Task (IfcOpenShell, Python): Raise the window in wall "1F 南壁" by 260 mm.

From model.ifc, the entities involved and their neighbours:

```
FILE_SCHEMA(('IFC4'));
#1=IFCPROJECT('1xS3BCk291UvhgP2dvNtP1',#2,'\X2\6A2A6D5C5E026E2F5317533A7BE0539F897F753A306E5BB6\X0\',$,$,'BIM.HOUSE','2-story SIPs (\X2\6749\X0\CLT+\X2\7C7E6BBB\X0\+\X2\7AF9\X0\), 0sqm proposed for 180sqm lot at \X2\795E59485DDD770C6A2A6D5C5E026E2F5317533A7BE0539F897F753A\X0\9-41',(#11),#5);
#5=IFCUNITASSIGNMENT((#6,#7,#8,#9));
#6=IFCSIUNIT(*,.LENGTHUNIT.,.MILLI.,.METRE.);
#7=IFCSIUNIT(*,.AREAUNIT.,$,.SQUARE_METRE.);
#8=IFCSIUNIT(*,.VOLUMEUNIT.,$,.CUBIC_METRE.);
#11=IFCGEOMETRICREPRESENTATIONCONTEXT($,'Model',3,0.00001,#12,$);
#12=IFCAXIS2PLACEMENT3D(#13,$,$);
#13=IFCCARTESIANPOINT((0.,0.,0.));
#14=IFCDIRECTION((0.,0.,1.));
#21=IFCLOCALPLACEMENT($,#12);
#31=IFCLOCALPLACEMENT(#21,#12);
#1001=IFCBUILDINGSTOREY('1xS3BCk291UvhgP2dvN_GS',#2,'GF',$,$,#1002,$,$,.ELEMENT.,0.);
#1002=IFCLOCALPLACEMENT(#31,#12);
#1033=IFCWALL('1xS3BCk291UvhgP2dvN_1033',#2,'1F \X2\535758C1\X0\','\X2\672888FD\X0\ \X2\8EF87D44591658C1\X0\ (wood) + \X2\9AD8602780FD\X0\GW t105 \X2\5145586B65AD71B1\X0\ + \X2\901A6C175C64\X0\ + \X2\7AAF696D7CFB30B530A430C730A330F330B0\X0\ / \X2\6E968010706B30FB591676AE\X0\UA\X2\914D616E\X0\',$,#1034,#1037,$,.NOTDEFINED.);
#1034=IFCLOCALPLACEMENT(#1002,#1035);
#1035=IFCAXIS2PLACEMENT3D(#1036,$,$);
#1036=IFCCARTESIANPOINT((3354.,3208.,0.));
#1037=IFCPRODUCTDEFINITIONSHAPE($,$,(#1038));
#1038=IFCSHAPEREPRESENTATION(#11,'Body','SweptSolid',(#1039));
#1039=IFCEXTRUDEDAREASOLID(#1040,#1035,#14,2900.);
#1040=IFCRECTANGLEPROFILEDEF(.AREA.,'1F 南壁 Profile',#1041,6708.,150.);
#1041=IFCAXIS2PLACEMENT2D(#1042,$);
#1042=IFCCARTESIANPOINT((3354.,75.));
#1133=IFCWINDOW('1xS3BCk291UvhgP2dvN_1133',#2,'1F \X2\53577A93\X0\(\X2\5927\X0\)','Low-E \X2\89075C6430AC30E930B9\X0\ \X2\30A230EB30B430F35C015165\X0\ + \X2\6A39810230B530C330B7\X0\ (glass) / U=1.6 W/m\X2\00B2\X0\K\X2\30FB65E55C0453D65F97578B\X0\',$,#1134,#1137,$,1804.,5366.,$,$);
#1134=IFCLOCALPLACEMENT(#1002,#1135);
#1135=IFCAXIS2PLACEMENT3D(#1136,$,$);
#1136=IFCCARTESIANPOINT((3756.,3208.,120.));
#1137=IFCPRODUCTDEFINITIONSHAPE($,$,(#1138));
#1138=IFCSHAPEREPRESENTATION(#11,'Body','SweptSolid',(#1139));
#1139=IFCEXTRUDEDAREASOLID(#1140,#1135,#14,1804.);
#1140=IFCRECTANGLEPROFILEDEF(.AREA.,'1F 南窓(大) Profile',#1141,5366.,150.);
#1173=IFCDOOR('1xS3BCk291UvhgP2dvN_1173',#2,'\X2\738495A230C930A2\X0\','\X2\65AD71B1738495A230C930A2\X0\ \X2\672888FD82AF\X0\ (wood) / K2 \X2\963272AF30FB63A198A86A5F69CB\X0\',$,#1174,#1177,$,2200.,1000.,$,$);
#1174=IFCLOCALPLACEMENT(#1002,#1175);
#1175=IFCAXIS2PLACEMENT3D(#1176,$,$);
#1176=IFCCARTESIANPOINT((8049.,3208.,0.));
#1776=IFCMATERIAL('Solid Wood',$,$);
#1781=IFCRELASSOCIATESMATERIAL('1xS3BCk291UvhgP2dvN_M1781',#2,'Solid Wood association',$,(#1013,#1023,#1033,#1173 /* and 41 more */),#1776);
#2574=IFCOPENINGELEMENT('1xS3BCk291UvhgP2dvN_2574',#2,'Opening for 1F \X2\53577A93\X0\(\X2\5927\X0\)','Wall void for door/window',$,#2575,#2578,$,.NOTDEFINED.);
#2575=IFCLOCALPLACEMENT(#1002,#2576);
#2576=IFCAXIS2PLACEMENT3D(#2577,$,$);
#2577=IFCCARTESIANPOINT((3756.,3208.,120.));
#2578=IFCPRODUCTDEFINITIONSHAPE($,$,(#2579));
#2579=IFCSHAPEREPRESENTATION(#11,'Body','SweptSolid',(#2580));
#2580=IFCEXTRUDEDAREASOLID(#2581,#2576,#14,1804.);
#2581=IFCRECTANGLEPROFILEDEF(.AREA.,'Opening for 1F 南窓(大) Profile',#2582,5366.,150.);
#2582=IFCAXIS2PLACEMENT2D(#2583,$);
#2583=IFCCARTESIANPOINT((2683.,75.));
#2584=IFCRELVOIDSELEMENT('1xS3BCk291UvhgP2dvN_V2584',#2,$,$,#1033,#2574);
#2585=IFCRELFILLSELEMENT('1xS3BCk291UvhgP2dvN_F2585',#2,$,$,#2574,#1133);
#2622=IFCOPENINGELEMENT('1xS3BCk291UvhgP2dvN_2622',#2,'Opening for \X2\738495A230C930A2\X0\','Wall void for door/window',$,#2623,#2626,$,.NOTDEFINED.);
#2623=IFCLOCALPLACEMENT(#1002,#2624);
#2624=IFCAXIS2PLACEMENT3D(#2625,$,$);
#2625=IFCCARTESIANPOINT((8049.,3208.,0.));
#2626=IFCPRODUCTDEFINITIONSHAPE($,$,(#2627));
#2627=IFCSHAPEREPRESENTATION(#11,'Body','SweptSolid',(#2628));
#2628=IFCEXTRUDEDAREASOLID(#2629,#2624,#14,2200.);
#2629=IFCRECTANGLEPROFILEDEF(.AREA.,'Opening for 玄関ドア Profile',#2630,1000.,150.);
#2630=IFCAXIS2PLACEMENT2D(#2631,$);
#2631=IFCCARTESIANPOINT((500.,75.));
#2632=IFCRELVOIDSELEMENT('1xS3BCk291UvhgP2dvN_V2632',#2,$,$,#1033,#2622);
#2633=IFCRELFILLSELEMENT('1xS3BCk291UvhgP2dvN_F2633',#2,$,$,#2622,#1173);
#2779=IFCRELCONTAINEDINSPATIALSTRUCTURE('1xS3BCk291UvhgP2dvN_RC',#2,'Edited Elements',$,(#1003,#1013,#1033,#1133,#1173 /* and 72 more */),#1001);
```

```python
import numpy as np
import ifcopenshell
import ifcopenshell.api.geometry
import ifcopenshell.util.placement
import ifcopenshell.util.unit

model = ifcopenshell.open("model.ifc")
unit_scale = ifcopenshell.util.unit.calculate_unit_scale(model)

window = model.by_guid("1xS3BCk291UvhgP2dvN_1133")
opening = window.FillsVoids[0].RelatingOpeningElement
dz = 0.26 / unit_scale

shift = np.array([0.0, 0.0, dz])
# The window is not placed relative to its opening, so move both.
for product in (opening, window):
    matrix = ifcopenshell.util.placement.get_local_placement(product.ObjectPlacement)
    matrix[:3, 3] += shift
    ifcopenshell.api.geometry.edit_object_placement(model, product=product, matrix=matrix, is_si=False)

print(f"moved by {dz * unit_scale:+.3f} m")

model.write("model-out.ifc")
```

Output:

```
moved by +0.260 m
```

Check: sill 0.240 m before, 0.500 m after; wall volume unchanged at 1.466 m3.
